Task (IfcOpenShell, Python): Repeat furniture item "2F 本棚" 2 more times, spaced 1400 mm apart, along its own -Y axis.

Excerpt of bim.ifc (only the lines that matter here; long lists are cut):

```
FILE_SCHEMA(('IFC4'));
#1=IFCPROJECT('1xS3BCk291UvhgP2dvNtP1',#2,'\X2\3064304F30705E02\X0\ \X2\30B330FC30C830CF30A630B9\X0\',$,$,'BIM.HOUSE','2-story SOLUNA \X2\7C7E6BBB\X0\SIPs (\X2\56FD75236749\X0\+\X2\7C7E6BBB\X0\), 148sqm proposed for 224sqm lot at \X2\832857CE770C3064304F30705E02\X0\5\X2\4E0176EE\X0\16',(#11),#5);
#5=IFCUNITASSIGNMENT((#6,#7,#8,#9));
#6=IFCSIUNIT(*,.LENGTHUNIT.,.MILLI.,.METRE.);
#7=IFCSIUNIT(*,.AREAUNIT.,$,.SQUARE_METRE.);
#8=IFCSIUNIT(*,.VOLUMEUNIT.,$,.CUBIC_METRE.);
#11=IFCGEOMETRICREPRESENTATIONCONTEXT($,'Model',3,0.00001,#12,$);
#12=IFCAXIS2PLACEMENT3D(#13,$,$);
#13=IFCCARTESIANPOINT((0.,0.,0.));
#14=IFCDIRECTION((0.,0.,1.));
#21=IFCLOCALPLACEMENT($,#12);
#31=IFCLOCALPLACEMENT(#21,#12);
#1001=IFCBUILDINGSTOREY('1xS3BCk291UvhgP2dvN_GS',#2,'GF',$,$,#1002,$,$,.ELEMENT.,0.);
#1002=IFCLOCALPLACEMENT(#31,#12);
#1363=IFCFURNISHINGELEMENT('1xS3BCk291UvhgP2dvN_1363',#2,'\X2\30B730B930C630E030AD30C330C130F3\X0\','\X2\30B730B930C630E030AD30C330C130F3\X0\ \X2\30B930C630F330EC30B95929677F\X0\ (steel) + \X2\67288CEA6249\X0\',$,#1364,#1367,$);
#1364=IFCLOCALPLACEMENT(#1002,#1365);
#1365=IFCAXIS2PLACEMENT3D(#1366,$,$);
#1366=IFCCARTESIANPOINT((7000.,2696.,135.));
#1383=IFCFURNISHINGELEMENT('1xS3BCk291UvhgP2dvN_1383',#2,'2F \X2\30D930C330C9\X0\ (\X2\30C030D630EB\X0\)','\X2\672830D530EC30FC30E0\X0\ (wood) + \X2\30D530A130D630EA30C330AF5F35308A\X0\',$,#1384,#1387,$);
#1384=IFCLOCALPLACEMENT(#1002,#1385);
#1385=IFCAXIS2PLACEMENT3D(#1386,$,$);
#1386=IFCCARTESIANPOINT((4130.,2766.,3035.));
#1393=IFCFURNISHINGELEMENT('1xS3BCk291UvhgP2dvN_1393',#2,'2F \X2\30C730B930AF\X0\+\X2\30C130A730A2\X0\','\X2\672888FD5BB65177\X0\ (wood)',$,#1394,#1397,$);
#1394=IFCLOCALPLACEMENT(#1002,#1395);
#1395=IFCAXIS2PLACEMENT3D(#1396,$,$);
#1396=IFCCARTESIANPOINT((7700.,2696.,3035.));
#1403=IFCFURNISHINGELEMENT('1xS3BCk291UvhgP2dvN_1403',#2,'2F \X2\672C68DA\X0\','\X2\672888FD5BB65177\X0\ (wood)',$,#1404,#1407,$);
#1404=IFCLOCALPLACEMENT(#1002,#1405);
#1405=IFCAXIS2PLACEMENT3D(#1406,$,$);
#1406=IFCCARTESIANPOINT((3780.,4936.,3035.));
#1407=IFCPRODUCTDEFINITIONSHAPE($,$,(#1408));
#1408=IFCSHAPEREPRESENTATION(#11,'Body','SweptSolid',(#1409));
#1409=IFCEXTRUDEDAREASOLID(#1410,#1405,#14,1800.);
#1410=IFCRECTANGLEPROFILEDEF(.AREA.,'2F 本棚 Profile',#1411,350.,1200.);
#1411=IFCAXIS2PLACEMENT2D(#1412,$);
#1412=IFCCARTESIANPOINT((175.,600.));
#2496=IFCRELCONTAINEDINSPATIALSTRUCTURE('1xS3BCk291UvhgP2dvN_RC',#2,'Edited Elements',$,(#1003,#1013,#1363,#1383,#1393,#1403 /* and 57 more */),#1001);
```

```python
import ifcopenshell
import ifcopenshell.api.geometry
import ifcopenshell.api.root
import ifcopenshell.util.element
import ifcopenshell.util.placement
import ifcopenshell.util.unit

model = ifcopenshell.open("bim.ifc")
unit_scale = ifcopenshell.util.unit.calculate_unit_scale(model)


def reuse_history(source, copy):
    """copy_class also copies each property set's owner history, people and application; keep the originals."""
    for rel in copy.IsDefinedBy:
        if rel.is_a("IfcRelDefinesByProperties") and (history := rel.RelatingPropertyDefinition.OwnerHistory):
            rel.RelatingPropertyDefinition.OwnerHistory = source.OwnerHistory
            ifcopenshell.util.element.remove_deep2(model, history)


source = model.by_id(1403)
base = ifcopenshell.util.placement.get_local_placement(source.ObjectPlacement)
step = -base[:3, 1] * 1.4 / unit_scale

for i in range(1, 3):
    copy = ifcopenshell.api.root.copy_class(model, product=source)
    copy.Representation = ifcopenshell.util.element.copy_deep(
        model, source.Representation, exclude=["IfcGeometricRepresentationContext", "IfcRepresentationMap"]
    )
    reuse_history(source, copy)
    matrix = base.copy()
    matrix[:3, 3] += i * step
    print("added at", matrix[:3, 3].round(3) + 0.0)
    ifcopenshell.api.geometry.edit_object_placement(model, product=copy, matrix=matrix, is_si=False)

model.write("bim-out.ifc")
```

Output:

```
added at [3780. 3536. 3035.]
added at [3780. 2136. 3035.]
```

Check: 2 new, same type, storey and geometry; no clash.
